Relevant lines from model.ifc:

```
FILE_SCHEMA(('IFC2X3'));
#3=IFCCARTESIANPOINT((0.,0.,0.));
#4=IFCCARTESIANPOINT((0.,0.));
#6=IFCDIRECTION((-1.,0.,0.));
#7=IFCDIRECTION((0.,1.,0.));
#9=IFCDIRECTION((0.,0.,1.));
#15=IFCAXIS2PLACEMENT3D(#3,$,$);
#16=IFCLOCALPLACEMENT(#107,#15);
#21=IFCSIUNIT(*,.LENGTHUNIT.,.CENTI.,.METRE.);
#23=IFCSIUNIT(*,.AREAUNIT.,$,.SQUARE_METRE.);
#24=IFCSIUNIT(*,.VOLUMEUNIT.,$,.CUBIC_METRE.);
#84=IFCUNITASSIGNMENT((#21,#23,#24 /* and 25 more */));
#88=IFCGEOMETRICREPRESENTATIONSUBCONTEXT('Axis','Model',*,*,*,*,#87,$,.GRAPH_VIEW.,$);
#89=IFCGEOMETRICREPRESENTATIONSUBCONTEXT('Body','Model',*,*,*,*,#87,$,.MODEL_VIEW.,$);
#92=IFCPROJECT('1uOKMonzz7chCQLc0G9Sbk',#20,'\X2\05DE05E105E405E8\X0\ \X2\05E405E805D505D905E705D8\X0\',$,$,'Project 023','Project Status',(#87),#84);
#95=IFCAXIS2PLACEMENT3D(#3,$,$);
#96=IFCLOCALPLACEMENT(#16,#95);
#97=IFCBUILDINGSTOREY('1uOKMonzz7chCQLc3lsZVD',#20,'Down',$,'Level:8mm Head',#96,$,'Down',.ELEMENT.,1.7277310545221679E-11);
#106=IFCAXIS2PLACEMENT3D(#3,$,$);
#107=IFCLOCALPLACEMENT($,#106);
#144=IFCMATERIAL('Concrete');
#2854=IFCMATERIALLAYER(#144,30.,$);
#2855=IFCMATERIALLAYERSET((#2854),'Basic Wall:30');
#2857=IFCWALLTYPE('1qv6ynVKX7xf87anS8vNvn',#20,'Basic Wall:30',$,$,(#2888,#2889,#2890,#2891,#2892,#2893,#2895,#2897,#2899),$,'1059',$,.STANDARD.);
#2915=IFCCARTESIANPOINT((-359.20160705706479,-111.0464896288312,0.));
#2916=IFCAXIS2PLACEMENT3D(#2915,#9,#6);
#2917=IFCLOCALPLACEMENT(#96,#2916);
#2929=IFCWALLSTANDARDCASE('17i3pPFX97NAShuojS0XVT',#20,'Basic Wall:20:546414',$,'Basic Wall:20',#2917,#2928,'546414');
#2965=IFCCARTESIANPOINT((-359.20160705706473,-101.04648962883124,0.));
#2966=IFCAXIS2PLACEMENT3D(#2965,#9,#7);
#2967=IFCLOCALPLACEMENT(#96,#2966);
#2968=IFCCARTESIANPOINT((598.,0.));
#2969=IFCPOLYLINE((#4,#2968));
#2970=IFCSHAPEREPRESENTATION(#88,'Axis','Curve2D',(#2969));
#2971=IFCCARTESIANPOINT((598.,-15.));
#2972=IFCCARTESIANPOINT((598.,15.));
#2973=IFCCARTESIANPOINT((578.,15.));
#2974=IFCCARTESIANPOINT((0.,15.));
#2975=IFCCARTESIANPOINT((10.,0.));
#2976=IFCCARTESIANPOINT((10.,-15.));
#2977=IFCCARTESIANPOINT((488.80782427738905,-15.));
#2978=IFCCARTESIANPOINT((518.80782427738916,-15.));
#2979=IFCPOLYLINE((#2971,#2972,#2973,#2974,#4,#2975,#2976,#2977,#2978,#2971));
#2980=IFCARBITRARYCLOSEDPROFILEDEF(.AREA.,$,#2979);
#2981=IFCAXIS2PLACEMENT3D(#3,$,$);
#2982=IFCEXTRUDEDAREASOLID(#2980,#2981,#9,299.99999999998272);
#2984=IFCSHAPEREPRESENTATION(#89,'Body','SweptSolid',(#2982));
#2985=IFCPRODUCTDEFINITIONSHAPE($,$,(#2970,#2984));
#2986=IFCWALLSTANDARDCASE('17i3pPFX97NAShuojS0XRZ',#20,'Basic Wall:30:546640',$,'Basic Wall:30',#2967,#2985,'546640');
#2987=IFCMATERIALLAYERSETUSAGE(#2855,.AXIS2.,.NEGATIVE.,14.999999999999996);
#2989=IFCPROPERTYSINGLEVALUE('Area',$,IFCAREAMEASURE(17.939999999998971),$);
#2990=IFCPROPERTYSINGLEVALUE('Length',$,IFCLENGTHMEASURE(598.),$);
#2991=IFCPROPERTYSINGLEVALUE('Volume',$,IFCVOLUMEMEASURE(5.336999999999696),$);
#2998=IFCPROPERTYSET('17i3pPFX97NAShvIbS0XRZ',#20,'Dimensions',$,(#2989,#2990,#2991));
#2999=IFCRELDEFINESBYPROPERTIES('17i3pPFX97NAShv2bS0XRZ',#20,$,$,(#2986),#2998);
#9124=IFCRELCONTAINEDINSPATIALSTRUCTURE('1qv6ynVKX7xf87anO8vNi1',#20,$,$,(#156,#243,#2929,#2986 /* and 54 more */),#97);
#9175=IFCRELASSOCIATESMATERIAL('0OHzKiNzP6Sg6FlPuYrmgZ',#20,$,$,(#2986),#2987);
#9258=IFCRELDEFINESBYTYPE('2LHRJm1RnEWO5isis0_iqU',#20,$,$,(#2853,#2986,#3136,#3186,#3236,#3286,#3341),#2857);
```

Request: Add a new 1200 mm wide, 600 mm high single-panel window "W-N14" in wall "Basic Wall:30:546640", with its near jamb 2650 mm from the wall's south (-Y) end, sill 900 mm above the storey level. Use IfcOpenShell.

```python
import numpy as np
import ifcopenshell
import ifcopenshell.api.feature
import ifcopenshell.api.geometry
import ifcopenshell.api.pset
import ifcopenshell.api.root
import ifcopenshell.api.spatial
import ifcopenshell.api.type
import ifcopenshell.geom
import ifcopenshell.util.element
import ifcopenshell.util.placement
import ifcopenshell.util.representation
import ifcopenshell.util.shape
import ifcopenshell.util.unit

model = ifcopenshell.open("model.ifc")
unit_scale = ifcopenshell.util.unit.calculate_unit_scale(model)
area_scale = ifcopenshell.util.unit.calculate_unit_scale(model, "AREAUNIT")
volume_scale = ifcopenshell.util.unit.calculate_unit_scale(model, "VOLUMEUNIT")
settings = ifcopenshell.geom.settings()


def volume(element):
    """Net volume in cubic metres, openings subtracted."""
    shape = ifcopenshell.geom.create_shape(settings, element)
    return ifcopenshell.util.shape.get_volume(shape.geometry)


wall = model.by_guid("17i3pPFX97NAShuojS0XRZ")
storey = ifcopenshell.util.element.get_container(wall, ifc_class="IfcBuildingStorey")
context = ifcopenshell.util.representation.get_context(model, "Model", "Body", "MODEL_VIEW")
before = volume(wall)

width, height, from_end, sill = 1.2, 0.6, 2.65, 0.9  # metres

# The wall runs along its own X axis, and the end named is its -X end.
wall_shape = ifcopenshell.geom.create_shape(settings, wall)
x, y, z = ifcopenshell.util.shape.get_vertices(wall_shape.geometry).T
start = x.min() + from_end
face, thickness = float(y.min()), float(y.max() - y.min())
wall_matrix = ifcopenshell.util.placement.get_local_placement(wall.ObjectPlacement)
level = ifcopenshell.util.placement.get_local_placement(storey.ObjectPlacement)[2, 3]


def in_wall(x, y):
    """Placement at x, y metres in the wall's axes, at sill height."""
    matrix = wall_matrix.copy()
    matrix[:, 3] = wall_matrix @ np.array([x / unit_scale, y / unit_scale, 0.0, 1.0])
    matrix[2, 3] = level + sill / unit_scale
    return matrix


# Opening: a box that overshoots both wall faces by 50 mm.
opening = ifcopenshell.api.root.create_entity(model, ifc_class="IfcOpeningElement")
box = ifcopenshell.api.geometry.add_wall_representation(
    model, context=context, length=width, height=height, thickness=thickness + 0.1
)
ifcopenshell.api.geometry.assign_representation(model, product=opening, representation=box)
ifcopenshell.api.geometry.edit_object_placement(model, product=opening, matrix=in_wall(start, face - 0.05), is_si=False)
ifcopenshell.api.feature.add_feature(model, feature=opening, element=wall)

window = ifcopenshell.api.root.create_entity(model, ifc_class="IfcWindow", name="W-N14")
window.OverallWidth, window.OverallHeight = width / unit_scale, height / unit_scale
body = ifcopenshell.api.geometry.add_window_representation(
    model,
    context=context,
    overall_width=window.OverallWidth,
    overall_height=window.OverallHeight,
    partition_type="SINGLE_PANEL",
)
ifcopenshell.api.geometry.assign_representation(model, product=window, representation=body)
ifcopenshell.api.spatial.assign_container(model, products=[window], relating_structure=storey)
fills = ifcopenshell.api.feature.add_filling(model, opening=opening, element=window)
fills.OwnerHistory = window.OwnerHistory  # required in IFC2X3

# IFC2X3 keeps the operation on the window style.
style = ifcopenshell.api.root.create_entity(model, ifc_class="IfcWindowStyle", name="W-N14")
style.OperationType, style.ConstructionType = "SINGLE_PANEL", "NOTDEFINED"
style.ParameterTakesPrecedence = style.Sizeable = False
ifcopenshell.api.type.assign_type(model, related_objects=[window], relating_type=style)

# Centre the window in the wall's thickness.
ifcopenshell.api.geometry.edit_object_placement(model, product=window, matrix=in_wall(start, face), is_si=False)
window_shape = ifcopenshell.geom.create_shape(settings, window)
depth = ifcopenshell.util.shape.get_vertices(window_shape.geometry)[:, 1]
offset = face + thickness / 2 - (depth.min() + depth.max()) / 2
ifcopenshell.api.geometry.edit_object_placement(model, product=window, matrix=in_wall(start, offset), is_si=False)

after = volume(wall)

# Update the wall's stored quantities.
pset = model.by_id(ifcopenshell.util.element.get_pset(wall, "Dimensions", should_inherit=False)["id"])
ifcopenshell.api.pset.edit_pset(model, pset=pset, properties={
    "Area": model.create_entity("IfcAreaMeasure", after / thickness / area_scale),
    "Volume": model.create_entity("IfcVolumeMeasure", after / volume_scale),
})

print(f"wall volume {before:.3f} -> {after:.3f} m3")

model.write("model_edited.ifc")
```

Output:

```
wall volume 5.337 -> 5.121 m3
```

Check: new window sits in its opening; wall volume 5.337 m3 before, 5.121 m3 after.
